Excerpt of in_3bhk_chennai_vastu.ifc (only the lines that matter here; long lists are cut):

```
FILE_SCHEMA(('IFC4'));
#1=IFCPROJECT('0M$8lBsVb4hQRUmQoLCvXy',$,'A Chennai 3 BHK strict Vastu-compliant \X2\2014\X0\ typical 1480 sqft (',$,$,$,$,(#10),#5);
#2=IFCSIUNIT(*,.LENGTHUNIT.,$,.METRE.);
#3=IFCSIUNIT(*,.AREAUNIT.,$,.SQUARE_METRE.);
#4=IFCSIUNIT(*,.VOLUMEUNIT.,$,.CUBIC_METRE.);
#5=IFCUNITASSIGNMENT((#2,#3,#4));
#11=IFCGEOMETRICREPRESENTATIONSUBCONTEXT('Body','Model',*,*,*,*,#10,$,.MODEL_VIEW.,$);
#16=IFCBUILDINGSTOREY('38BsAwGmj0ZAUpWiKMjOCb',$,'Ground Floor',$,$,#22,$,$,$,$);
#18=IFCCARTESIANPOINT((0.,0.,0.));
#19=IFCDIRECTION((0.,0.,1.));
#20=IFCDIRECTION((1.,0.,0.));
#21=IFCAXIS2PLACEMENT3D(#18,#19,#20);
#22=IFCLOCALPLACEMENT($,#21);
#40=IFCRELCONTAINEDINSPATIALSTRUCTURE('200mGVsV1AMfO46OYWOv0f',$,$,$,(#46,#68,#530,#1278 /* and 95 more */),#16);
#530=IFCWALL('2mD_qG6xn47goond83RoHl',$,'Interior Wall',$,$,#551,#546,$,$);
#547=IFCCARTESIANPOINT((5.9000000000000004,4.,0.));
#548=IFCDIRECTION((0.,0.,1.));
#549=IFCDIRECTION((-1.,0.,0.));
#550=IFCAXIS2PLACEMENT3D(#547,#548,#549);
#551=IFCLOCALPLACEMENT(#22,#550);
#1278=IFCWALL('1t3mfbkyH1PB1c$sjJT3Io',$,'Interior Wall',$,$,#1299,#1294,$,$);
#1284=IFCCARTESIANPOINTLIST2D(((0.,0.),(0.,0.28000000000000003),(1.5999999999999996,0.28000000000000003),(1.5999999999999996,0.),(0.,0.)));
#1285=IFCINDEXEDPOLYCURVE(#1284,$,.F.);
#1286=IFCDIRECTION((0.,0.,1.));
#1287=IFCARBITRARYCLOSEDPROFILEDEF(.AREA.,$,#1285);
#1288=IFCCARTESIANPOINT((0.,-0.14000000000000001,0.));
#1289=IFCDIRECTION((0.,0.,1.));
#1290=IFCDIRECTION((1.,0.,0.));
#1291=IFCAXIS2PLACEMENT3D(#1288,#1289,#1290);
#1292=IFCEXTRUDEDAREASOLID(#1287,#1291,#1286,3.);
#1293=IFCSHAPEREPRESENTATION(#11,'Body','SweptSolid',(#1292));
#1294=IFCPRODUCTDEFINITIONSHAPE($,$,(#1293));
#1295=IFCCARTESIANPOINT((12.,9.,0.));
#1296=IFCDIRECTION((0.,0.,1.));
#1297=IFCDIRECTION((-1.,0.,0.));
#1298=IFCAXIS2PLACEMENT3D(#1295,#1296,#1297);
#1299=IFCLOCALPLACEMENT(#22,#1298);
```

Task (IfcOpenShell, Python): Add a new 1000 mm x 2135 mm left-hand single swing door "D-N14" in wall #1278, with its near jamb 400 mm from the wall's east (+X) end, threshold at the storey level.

```python
import numpy as np
import ifcopenshell
import ifcopenshell.api.feature
import ifcopenshell.api.geometry
import ifcopenshell.api.root
import ifcopenshell.api.spatial
import ifcopenshell.geom
import ifcopenshell.util.element
import ifcopenshell.util.placement
import ifcopenshell.util.representation
import ifcopenshell.util.shape
import ifcopenshell.util.unit

model = ifcopenshell.open("in_3bhk_chennai_vastu.ifc")
unit_scale = ifcopenshell.util.unit.calculate_unit_scale(model)
settings = ifcopenshell.geom.settings()


def volume(element):
    """Net volume in cubic metres, openings subtracted."""
    shape = ifcopenshell.geom.create_shape(settings, element)
    return ifcopenshell.util.shape.get_volume(shape.geometry)


wall = model.by_guid("1t3mfbkyH1PB1c$sjJT3Io")
storey = ifcopenshell.util.element.get_container(wall, ifc_class="IfcBuildingStorey")
context = ifcopenshell.util.representation.get_context(model, "Model", "Body", "MODEL_VIEW")
before = volume(wall)

width, height, from_end, sill = 1, 2.135, 0.4, 0.0  # metres

# The wall runs along its own X axis, and the end named is its -X end.
wall_shape = ifcopenshell.geom.create_shape(settings, wall)
x, y, z = ifcopenshell.util.shape.get_vertices(wall_shape.geometry).T
start = x.min() + from_end
face, thickness = float(y.min()), float(y.max() - y.min())
wall_matrix = ifcopenshell.util.placement.get_local_placement(wall.ObjectPlacement)
level = ifcopenshell.util.placement.get_local_placement(storey.ObjectPlacement)[2, 3]


def in_wall(x, y):
    """Placement at x, y metres in the wall's axes, at sill height."""
    matrix = wall_matrix.copy()
    matrix[:, 3] = wall_matrix @ np.array([x / unit_scale, y / unit_scale, 0.0, 1.0])
    matrix[2, 3] = level + sill / unit_scale
    return matrix


# Opening: a box that overshoots both wall faces by 50 mm.
opening = ifcopenshell.api.root.create_entity(model, ifc_class="IfcOpeningElement", predefined_type="OPENING")
box = ifcopenshell.api.geometry.add_wall_representation(
    model, context=context, length=width, height=height, thickness=thickness + 0.1
)
ifcopenshell.api.geometry.assign_representation(model, product=opening, representation=box)
ifcopenshell.api.geometry.edit_object_placement(model, product=opening, matrix=in_wall(start, face - 0.05), is_si=False)
ifcopenshell.api.feature.add_feature(model, feature=opening, element=wall)

door = ifcopenshell.api.root.create_entity(model, ifc_class="IfcDoor", name="D-N14", predefined_type="DOOR")
door.OverallWidth, door.OverallHeight = width / unit_scale, height / unit_scale
door.OperationType = "SINGLE_SWING_LEFT"
body = ifcopenshell.api.geometry.add_door_representation(
    model,
    context=context,
    overall_width=door.OverallWidth,
    overall_height=door.OverallHeight,
    operation_type="SINGLE_SWING_LEFT",
    lining_properties={"LiningDepth": thickness / unit_scale, "ThresholdDepth": thickness / unit_scale},
)
ifcopenshell.api.geometry.assign_representation(model, product=door, representation=body)
ifcopenshell.api.spatial.assign_container(model, products=[door], relating_structure=storey)
ifcopenshell.api.feature.add_filling(model, opening=opening, element=door)

# The lining spans the wall, so the door starts at the wall face.
ifcopenshell.api.geometry.edit_object_placement(model, product=door, matrix=in_wall(start, face), is_si=False)

after = volume(wall)

print(f"wall volume {before:.3f} -> {after:.3f} m3")

model.write("in_3bhk_chennai_vastu_v2.ifc")
```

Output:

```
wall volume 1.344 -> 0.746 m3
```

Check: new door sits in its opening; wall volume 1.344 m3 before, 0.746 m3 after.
